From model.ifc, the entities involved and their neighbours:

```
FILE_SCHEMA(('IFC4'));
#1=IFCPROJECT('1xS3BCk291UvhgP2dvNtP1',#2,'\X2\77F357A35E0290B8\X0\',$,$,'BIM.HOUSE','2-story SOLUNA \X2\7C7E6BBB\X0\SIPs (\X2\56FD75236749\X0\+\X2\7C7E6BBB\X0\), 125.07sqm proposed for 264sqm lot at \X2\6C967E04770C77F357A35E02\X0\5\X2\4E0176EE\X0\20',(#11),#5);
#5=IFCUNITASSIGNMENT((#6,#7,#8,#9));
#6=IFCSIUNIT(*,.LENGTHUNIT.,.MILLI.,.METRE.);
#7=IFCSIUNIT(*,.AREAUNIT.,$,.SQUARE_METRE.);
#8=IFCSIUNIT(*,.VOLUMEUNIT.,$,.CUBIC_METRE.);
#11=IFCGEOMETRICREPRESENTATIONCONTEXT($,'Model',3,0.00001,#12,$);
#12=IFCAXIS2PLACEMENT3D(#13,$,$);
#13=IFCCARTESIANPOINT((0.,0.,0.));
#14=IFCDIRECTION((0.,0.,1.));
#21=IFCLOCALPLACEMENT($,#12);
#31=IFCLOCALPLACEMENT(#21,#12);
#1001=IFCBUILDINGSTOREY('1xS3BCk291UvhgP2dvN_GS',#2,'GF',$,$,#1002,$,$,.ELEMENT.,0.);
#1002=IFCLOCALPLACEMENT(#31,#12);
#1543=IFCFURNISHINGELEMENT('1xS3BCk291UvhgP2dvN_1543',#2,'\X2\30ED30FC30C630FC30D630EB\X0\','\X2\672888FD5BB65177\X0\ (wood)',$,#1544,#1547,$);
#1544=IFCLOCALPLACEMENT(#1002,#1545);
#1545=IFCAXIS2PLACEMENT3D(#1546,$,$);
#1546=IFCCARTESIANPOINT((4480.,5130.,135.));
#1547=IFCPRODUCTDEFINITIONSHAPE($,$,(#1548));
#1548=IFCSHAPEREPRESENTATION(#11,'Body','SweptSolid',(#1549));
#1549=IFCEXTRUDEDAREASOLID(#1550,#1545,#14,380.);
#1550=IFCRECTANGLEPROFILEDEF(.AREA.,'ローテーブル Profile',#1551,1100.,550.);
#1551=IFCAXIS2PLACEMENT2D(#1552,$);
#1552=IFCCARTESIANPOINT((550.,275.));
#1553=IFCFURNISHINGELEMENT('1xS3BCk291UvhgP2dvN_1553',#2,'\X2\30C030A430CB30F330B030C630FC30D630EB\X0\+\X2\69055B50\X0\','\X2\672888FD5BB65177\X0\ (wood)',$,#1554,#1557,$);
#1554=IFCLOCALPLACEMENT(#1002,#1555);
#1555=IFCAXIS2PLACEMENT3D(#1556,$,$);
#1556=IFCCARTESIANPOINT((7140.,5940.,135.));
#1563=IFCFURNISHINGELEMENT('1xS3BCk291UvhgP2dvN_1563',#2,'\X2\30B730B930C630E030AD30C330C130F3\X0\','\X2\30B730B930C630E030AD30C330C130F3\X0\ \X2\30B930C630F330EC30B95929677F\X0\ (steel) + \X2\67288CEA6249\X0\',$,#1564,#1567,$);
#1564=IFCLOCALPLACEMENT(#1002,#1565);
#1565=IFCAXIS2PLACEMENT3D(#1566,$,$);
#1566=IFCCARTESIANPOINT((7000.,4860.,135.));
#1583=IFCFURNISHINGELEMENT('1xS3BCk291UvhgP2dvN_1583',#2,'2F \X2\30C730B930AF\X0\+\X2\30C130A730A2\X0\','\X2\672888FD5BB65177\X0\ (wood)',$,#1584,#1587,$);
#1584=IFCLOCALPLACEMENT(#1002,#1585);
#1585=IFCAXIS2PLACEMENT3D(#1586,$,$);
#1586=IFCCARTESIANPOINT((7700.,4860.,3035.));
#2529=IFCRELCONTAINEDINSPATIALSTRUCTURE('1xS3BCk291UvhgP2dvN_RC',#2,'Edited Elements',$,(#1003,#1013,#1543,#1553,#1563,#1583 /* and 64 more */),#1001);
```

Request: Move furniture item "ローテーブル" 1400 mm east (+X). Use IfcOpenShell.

```python
import ifcopenshell
import ifcopenshell.api.geometry
import ifcopenshell.util.placement
import ifcopenshell.util.unit

model = ifcopenshell.open("model.ifc")
unit_scale = ifcopenshell.util.unit.calculate_unit_scale(model)

item = model.by_guid("1xS3BCk291UvhgP2dvN_1543")
matrix = ifcopenshell.util.placement.get_local_placement(item.ObjectPlacement)
matrix[0, 3] += 1.4 / unit_scale
ifcopenshell.api.geometry.edit_object_placement(model, product=item, matrix=matrix, is_si=False)

print(ifcopenshell.util.placement.get_local_placement(item.ObjectPlacement).round(3) + 0.0)

model.write("model-out.ifc")
```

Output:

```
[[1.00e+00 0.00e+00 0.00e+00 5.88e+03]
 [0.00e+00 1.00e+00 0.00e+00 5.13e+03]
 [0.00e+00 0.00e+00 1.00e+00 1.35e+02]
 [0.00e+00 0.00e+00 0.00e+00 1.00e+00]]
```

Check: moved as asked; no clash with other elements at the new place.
